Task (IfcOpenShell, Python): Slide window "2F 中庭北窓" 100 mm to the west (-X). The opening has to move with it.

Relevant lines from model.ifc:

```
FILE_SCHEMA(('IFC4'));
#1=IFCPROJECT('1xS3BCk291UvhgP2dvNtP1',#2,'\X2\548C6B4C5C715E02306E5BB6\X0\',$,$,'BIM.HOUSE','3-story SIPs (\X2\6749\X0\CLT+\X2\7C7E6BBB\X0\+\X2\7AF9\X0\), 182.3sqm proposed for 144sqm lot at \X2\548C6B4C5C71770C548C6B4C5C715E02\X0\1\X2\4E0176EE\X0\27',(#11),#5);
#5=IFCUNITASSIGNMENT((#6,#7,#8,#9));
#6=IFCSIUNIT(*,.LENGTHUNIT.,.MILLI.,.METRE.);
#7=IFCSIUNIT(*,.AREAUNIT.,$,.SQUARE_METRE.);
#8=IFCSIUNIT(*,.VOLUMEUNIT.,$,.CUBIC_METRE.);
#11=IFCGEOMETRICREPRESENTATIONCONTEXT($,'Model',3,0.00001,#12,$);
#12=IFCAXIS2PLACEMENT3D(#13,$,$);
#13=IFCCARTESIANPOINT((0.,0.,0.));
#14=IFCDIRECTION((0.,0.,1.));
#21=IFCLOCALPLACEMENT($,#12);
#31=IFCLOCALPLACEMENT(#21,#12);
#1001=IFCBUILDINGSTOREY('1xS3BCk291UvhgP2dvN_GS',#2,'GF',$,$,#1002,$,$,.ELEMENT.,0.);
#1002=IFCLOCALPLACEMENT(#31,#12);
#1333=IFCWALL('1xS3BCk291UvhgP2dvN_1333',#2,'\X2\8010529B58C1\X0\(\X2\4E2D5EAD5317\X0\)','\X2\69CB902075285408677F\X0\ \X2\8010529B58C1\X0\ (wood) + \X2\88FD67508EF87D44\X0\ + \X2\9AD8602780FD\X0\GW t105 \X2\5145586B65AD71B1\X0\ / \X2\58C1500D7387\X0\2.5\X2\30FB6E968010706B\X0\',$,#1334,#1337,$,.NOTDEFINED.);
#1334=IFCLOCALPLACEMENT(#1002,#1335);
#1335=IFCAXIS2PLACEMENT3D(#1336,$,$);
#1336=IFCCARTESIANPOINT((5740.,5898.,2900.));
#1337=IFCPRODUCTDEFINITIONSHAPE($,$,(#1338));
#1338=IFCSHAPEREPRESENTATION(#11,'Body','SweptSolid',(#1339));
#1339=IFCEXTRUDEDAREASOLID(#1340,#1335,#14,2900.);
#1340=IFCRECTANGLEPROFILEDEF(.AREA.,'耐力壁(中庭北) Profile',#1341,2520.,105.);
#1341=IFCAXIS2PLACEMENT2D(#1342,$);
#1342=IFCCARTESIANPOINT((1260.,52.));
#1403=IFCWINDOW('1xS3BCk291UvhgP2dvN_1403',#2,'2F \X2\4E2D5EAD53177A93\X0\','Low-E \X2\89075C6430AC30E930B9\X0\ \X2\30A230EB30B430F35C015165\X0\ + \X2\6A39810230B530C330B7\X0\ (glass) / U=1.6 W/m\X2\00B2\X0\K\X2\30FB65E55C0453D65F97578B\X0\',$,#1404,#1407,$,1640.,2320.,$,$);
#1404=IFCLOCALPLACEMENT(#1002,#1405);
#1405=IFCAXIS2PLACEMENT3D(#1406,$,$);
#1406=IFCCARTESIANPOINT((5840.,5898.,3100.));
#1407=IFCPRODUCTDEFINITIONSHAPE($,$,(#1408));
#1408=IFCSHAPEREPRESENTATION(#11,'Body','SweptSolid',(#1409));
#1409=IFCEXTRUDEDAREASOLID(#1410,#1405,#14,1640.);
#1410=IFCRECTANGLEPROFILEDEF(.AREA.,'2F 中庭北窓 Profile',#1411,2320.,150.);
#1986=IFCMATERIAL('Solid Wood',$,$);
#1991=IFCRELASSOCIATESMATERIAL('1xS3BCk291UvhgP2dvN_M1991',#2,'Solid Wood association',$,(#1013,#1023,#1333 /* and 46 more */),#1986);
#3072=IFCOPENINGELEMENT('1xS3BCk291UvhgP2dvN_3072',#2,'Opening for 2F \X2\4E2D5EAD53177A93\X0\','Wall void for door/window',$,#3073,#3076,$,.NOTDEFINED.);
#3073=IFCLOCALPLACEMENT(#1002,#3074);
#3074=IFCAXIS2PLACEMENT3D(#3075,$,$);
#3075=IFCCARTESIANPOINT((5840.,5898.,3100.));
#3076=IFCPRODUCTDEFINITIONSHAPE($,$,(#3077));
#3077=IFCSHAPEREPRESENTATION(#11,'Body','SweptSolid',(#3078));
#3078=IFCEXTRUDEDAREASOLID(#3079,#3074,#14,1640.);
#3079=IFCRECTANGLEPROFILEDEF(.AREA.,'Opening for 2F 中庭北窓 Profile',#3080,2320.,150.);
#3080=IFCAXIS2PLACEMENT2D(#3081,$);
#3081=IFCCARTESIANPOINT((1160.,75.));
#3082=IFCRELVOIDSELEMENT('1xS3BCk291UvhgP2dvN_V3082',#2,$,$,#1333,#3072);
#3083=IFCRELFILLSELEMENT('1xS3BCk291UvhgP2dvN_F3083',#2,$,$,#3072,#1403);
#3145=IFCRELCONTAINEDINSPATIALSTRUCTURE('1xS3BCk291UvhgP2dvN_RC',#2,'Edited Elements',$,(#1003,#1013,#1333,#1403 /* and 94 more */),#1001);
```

```python
import ifcopenshell
import ifcopenshell.api.geometry
import ifcopenshell.util.placement
import ifcopenshell.util.unit

model = ifcopenshell.open("model.ifc")
unit_scale = ifcopenshell.util.unit.calculate_unit_scale(model)

window = model.by_guid("1xS3BCk291UvhgP2dvN_1403")
opening = window.FillsVoids[0].RelatingOpeningElement
wall = opening.VoidsElements[0].RelatingBuildingElement

wall_matrix = ifcopenshell.util.placement.get_local_placement(wall.ObjectPlacement)
shift = wall_matrix[:3, 0] * -0.1 / unit_scale
before = ifcopenshell.util.placement.get_local_placement(window.ObjectPlacement)[:3, 3].copy()

# The window is not placed relative to its opening, so move both.
for product in (opening, window):
    matrix = ifcopenshell.util.placement.get_local_placement(product.ObjectPlacement)
    matrix[:3, 3] += shift
    ifcopenshell.api.geometry.edit_object_placement(model, product=product, matrix=matrix, is_si=False)

after = ifcopenshell.util.placement.get_local_placement(window.ObjectPlacement)[:3, 3]
print("window moved by", (after - before).round(3) + 0.0)

model.write("model-out.ifc")
```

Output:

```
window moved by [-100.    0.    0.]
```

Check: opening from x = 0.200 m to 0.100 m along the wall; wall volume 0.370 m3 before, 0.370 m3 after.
